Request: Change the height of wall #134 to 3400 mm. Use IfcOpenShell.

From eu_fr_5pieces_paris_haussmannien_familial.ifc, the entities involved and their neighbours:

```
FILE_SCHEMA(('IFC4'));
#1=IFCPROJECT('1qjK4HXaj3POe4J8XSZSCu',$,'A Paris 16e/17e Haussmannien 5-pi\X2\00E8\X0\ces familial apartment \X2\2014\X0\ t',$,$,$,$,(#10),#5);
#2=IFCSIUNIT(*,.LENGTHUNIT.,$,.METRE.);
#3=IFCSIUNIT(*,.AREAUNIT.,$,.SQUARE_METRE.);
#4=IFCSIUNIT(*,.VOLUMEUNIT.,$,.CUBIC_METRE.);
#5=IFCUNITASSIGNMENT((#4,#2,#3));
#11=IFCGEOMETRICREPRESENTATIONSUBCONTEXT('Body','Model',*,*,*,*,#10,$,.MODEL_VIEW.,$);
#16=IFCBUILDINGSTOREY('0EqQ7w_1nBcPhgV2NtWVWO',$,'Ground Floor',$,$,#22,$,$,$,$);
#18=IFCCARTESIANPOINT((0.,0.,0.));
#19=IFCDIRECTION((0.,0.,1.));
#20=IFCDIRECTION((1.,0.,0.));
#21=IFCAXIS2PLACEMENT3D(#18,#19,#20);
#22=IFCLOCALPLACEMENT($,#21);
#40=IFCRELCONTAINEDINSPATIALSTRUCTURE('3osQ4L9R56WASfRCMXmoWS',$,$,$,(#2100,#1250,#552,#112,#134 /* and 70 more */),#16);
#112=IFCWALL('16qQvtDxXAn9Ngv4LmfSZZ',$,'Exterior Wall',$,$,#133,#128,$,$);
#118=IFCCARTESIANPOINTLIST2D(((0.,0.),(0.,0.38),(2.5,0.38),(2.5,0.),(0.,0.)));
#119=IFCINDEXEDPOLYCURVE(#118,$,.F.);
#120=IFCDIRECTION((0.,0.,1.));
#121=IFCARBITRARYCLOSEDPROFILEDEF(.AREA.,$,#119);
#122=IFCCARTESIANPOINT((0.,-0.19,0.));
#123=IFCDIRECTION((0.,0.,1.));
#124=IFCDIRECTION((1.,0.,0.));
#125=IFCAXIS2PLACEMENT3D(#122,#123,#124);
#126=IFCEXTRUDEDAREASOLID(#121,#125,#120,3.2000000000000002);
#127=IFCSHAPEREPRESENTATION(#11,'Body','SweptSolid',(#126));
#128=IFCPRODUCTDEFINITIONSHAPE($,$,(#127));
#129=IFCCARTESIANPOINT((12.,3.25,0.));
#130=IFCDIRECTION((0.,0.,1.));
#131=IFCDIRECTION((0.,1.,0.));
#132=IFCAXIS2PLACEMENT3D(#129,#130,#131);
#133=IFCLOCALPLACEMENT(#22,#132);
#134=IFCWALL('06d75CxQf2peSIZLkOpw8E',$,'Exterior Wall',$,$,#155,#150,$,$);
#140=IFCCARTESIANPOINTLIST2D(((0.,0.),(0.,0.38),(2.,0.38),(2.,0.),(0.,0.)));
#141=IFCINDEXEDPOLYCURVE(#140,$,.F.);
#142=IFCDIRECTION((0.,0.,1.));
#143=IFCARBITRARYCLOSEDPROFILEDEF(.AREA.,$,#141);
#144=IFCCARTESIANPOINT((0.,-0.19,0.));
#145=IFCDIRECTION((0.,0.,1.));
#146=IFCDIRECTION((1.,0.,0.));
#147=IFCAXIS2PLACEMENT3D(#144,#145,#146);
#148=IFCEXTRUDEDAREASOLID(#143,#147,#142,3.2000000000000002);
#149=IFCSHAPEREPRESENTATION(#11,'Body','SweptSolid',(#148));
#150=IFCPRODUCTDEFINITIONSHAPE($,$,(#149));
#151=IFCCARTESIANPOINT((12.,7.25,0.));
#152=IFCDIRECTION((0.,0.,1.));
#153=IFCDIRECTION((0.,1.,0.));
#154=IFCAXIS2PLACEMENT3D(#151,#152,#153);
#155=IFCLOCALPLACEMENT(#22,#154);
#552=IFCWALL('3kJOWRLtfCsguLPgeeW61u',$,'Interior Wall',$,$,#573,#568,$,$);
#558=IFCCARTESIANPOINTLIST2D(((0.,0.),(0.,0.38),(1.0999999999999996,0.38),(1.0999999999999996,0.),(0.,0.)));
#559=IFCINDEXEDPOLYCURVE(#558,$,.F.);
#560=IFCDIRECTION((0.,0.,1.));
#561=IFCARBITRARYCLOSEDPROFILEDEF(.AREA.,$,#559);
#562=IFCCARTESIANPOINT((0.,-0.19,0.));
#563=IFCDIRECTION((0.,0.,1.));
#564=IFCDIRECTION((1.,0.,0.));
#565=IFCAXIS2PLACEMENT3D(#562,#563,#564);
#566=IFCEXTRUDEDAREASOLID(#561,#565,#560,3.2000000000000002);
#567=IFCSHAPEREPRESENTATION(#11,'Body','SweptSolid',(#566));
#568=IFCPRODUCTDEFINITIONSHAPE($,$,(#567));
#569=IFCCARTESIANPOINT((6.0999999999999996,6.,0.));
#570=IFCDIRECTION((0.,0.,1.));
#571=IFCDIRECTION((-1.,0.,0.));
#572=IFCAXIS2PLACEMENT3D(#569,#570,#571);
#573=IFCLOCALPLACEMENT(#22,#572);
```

```python
import ifcopenshell
import ifcopenshell.geom
import ifcopenshell.util.representation
import ifcopenshell.util.shape
import ifcopenshell.util.unit

model = ifcopenshell.open("eu_fr_5pieces_paris_haussmannien_familial.ifc")
unit_scale = ifcopenshell.util.unit.calculate_unit_scale(model)
settings = ifcopenshell.geom.settings()


def volume(element):
    """Net volume in cubic metres, openings subtracted."""
    shape = ifcopenshell.geom.create_shape(settings, element)
    return ifcopenshell.util.shape.get_volume(shape.geometry)


wall = model.by_guid("06d75CxQf2peSIZLkOpw8E")
before = volume(wall)

body = ifcopenshell.util.representation.get_representation(wall, "Model", "Body")
solid = body.Items[0]
old_height = solid.Depth
solid.Depth = 3.4 / unit_scale
after = volume(wall)

print(f"height {old_height:g} -> {solid.Depth:g}, volume {before:.3f} -> {after:.3f} m3")

model.write("eu_fr_5pieces_paris_haussmannien_familial_updated.ifc")
```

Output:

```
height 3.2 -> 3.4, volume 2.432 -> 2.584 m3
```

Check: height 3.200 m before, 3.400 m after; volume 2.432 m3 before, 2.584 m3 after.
